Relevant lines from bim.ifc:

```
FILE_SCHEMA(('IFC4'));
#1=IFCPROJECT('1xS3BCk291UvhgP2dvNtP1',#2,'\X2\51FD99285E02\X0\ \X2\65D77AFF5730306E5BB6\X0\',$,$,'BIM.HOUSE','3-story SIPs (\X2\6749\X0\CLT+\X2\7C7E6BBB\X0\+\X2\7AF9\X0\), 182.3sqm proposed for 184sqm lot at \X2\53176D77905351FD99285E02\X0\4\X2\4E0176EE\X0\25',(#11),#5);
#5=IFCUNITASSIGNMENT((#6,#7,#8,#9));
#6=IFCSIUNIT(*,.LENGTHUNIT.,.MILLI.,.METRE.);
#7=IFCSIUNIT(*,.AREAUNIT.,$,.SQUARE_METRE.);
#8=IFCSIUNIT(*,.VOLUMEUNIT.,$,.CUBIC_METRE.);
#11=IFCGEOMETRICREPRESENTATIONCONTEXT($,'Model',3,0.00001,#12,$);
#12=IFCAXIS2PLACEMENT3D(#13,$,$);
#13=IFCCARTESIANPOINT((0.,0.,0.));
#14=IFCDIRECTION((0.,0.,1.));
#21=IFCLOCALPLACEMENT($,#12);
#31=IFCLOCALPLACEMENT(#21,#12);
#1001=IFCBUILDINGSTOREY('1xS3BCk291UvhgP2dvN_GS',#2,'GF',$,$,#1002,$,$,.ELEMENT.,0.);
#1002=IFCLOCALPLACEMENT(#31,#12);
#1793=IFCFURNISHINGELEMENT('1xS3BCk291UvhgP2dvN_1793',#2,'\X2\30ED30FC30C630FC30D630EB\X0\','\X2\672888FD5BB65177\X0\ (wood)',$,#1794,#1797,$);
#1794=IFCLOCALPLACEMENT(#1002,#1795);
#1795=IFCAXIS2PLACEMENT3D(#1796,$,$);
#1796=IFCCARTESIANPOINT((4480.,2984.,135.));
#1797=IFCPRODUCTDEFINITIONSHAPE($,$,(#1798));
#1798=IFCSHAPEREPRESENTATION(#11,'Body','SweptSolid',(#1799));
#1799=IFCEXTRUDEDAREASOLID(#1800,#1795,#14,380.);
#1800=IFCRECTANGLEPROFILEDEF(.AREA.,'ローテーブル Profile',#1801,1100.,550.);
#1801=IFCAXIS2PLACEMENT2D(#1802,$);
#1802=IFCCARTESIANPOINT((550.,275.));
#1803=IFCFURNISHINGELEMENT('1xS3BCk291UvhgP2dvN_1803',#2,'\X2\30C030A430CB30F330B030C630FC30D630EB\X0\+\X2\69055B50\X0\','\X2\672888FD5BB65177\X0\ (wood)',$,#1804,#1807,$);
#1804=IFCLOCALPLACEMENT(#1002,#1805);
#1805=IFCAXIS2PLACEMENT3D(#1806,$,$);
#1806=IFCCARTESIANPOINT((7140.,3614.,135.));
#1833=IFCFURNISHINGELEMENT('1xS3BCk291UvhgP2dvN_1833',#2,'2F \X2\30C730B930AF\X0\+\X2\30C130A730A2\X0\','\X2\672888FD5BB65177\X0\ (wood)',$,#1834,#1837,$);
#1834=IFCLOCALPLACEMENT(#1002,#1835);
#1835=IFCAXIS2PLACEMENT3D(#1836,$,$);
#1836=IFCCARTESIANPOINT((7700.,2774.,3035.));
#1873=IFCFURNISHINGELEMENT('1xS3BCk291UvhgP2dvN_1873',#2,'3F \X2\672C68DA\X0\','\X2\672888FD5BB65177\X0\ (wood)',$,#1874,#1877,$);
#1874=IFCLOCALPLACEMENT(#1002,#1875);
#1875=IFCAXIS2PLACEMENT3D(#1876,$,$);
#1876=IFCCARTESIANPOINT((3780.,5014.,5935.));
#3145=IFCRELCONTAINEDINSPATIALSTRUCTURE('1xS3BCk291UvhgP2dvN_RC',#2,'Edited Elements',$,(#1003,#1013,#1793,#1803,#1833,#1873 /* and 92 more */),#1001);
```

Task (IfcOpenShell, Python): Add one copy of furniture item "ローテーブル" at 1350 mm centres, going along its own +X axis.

```python
import ifcopenshell
import ifcopenshell.api.geometry
import ifcopenshell.api.root
import ifcopenshell.util.element
import ifcopenshell.util.placement

model = ifcopenshell.open("bim.ifc")


def reuse_history(source, copy):
    """copy_class also copies each property set's owner history, people and application; keep the originals."""
    for rel in copy.IsDefinedBy:
        if rel.is_a("IfcRelDefinesByProperties") and (history := rel.RelatingPropertyDefinition.OwnerHistory):
            rel.RelatingPropertyDefinition.OwnerHistory = source.OwnerHistory
            ifcopenshell.util.element.remove_deep2(model, history)


source = model.by_guid("1xS3BCk291UvhgP2dvN_1793")
base = ifcopenshell.util.placement.get_local_placement(source.ObjectPlacement)
step = base[:3, 0] * 1350.0

for i in range(1, 2):
    copy = ifcopenshell.api.root.copy_class(model, product=source)
    copy.Representation = ifcopenshell.util.element.copy_deep(
        model, source.Representation, exclude=["IfcGeometricRepresentationContext", "IfcRepresentationMap"]
    )
    reuse_history(source, copy)
    matrix = base.copy()
    matrix[:3, 3] += i * step
    print("added at", matrix[:3, 3].round(3) + 0.0)
    ifcopenshell.api.geometry.edit_object_placement(model, product=copy, matrix=matrix, is_si=False)

model.write("bim_rev.ifc")
```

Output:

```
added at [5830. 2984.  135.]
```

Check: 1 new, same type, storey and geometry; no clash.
